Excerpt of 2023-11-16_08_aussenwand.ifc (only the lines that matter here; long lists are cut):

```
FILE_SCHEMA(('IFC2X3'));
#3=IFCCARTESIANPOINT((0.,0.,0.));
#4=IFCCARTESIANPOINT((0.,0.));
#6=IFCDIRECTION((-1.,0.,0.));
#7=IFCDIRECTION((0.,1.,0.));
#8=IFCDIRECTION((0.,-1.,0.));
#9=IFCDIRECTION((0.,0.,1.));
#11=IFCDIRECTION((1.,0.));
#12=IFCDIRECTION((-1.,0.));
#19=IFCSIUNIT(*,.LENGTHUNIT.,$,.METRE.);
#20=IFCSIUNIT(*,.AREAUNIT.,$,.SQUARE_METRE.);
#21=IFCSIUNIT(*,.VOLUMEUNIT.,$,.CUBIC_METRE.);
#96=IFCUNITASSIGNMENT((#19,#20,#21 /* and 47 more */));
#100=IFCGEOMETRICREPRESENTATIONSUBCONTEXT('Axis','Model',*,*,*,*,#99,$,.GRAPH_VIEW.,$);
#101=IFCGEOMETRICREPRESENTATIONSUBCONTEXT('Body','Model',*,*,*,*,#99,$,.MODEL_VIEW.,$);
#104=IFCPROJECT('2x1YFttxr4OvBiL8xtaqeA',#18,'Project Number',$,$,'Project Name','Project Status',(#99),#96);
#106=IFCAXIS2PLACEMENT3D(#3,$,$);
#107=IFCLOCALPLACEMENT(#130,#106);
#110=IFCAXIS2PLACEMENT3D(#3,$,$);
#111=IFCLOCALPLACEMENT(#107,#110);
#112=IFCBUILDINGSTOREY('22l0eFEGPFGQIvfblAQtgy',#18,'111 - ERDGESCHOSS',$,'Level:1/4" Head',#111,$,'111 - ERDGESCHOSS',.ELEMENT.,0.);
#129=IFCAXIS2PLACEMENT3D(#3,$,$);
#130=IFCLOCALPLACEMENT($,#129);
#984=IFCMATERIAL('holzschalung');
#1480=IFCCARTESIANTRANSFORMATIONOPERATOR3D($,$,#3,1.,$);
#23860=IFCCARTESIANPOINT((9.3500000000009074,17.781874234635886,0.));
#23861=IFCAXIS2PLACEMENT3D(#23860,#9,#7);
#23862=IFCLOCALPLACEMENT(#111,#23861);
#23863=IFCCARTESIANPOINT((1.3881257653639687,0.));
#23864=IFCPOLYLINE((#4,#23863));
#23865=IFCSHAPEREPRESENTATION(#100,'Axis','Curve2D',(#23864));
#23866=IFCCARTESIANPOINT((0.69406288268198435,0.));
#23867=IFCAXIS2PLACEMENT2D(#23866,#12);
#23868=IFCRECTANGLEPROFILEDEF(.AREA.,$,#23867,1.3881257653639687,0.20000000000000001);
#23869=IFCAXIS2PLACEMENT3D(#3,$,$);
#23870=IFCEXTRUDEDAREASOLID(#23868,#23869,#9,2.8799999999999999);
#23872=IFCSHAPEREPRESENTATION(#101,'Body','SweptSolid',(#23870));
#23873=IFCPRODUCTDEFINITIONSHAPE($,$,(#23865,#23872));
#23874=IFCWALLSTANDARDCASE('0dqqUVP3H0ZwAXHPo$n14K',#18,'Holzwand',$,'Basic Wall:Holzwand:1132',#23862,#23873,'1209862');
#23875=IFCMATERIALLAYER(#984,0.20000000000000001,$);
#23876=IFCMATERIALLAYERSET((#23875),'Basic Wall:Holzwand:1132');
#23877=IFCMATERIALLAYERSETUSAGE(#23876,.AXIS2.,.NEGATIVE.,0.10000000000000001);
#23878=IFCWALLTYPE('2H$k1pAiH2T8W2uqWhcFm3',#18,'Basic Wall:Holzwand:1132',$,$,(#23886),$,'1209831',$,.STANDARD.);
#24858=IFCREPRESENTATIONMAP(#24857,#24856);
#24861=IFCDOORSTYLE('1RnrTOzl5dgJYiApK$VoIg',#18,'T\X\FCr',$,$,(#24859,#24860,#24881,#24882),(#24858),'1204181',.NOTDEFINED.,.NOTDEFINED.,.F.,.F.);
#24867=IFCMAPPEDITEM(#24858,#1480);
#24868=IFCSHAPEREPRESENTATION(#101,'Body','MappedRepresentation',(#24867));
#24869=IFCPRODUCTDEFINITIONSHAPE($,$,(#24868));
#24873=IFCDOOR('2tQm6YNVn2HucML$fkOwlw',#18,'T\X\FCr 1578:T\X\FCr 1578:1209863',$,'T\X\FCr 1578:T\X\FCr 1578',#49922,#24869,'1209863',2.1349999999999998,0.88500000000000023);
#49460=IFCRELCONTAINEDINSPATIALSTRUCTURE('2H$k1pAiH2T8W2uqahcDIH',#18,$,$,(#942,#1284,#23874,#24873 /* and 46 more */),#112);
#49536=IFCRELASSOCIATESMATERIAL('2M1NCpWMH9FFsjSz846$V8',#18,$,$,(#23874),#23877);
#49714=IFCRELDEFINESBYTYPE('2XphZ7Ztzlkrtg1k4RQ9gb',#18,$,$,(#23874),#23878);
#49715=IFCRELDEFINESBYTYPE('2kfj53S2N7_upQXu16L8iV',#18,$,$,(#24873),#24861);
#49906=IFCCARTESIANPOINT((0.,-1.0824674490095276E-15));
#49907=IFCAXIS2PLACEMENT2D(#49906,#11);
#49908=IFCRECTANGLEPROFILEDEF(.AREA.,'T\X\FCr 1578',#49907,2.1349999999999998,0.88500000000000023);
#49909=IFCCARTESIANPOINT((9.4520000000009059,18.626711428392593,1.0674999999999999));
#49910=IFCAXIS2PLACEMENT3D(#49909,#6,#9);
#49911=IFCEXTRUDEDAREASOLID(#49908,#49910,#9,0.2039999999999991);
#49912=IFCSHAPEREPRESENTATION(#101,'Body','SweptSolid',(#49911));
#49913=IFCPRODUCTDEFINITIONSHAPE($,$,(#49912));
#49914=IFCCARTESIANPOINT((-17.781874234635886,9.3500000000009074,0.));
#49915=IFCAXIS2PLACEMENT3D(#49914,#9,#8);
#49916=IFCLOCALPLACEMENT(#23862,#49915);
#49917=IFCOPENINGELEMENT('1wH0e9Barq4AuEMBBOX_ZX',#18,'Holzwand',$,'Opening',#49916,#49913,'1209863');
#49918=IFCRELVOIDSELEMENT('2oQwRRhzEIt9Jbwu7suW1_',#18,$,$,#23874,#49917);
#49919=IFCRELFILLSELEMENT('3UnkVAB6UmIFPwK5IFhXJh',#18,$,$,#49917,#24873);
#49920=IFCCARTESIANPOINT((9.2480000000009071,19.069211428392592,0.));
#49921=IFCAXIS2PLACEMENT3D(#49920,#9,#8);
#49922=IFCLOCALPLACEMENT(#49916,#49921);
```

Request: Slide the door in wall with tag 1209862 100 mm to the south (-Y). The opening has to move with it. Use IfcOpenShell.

```python
import ifcopenshell
import ifcopenshell.api.geometry
import ifcopenshell.util.placement

model = ifcopenshell.open("2023-11-16_08_aussenwand.ifc")

door = model.by_guid("2tQm6YNVn2HucML$fkOwlw")
opening = door.FillsVoids[0].RelatingOpeningElement
wall = opening.VoidsElements[0].RelatingBuildingElement

wall_matrix = ifcopenshell.util.placement.get_local_placement(wall.ObjectPlacement)
shift = wall_matrix[:3, 0] * -0.1
before = ifcopenshell.util.placement.get_local_placement(door.ObjectPlacement)[:3, 3].copy()

# The door is placed relative to its opening, so it follows when the opening moves.
matrix = ifcopenshell.util.placement.get_local_placement(opening.ObjectPlacement)
matrix[:3, 3] += shift
ifcopenshell.api.geometry.edit_object_placement(
    model, product=opening, matrix=matrix, is_si=False, should_transform_children=True
)

after = ifcopenshell.util.placement.get_local_placement(door.ObjectPlacement)[:3, 3]
print("door moved by", (after - before).round(3) + 0.0)

model.write("2023-11-16_08_aussenwand-out.ifc")
```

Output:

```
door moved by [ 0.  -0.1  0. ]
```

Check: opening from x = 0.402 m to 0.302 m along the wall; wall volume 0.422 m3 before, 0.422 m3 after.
